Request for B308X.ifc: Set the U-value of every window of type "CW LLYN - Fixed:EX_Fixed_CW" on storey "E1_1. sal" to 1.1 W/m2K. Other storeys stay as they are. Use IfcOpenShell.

First a look at what the model holds.

```python
import ifcopenshell
import ifcopenshell.util.element

model = ifcopenshell.open("B308X.ifc")
print(model.schema)
storey = next(s for s in model.by_type("IfcBuildingStorey") if s.Name == "E1_1. sal")
windows = [e for e in ifcopenshell.util.element.get_decomposition(storey) if e.is_a("IfcWindow")]
seen = {}
for e in windows:
    element_type = ifcopenshell.util.element.get_type(e)
    key = (element_type.Name if element_type != e and element_type else None, ifcopenshell.util.element.get_pset(e, "Pset_WindowCommon", "ThermalTransmittance"))
    seen[key] = seen.get(key, 0) + 1
for (name, value), count in sorted(seen.items(), key=str):
    print(count, "x", name, "|", value)
```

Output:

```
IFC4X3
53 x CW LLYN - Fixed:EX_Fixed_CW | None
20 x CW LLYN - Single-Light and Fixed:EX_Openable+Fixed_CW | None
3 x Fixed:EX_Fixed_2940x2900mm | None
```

```python
import ifcopenshell
import ifcopenshell.api.pset
import ifcopenshell.util.element

model = ifcopenshell.open("B308X.ifc")

storey = next(s for s in model.by_type("IfcBuildingStorey") if s.Name == "E1_1. sal")
windows = [e for e in ifcopenshell.util.element.get_decomposition(storey) if e.is_a("IfcWindow")]

count = 0
for e in windows:
    element_type = ifcopenshell.util.element.get_type(e)
    if element_type in (None, e) or element_type.Name != "CW LLYN - Fixed:EX_Fixed_CW":
        continue
    # add_pset returns the element's existing set when there is one.
    pset = ifcopenshell.api.pset.add_pset(model, product=e, name="Pset_WindowCommon")
    ifcopenshell.api.pset.edit_pset(model, pset=pset, properties={"ThermalTransmittance": 1.1})
    count += 1

print(count, "windows updated")

model.write("B308X_rev.ifc")
```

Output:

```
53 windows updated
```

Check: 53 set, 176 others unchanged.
